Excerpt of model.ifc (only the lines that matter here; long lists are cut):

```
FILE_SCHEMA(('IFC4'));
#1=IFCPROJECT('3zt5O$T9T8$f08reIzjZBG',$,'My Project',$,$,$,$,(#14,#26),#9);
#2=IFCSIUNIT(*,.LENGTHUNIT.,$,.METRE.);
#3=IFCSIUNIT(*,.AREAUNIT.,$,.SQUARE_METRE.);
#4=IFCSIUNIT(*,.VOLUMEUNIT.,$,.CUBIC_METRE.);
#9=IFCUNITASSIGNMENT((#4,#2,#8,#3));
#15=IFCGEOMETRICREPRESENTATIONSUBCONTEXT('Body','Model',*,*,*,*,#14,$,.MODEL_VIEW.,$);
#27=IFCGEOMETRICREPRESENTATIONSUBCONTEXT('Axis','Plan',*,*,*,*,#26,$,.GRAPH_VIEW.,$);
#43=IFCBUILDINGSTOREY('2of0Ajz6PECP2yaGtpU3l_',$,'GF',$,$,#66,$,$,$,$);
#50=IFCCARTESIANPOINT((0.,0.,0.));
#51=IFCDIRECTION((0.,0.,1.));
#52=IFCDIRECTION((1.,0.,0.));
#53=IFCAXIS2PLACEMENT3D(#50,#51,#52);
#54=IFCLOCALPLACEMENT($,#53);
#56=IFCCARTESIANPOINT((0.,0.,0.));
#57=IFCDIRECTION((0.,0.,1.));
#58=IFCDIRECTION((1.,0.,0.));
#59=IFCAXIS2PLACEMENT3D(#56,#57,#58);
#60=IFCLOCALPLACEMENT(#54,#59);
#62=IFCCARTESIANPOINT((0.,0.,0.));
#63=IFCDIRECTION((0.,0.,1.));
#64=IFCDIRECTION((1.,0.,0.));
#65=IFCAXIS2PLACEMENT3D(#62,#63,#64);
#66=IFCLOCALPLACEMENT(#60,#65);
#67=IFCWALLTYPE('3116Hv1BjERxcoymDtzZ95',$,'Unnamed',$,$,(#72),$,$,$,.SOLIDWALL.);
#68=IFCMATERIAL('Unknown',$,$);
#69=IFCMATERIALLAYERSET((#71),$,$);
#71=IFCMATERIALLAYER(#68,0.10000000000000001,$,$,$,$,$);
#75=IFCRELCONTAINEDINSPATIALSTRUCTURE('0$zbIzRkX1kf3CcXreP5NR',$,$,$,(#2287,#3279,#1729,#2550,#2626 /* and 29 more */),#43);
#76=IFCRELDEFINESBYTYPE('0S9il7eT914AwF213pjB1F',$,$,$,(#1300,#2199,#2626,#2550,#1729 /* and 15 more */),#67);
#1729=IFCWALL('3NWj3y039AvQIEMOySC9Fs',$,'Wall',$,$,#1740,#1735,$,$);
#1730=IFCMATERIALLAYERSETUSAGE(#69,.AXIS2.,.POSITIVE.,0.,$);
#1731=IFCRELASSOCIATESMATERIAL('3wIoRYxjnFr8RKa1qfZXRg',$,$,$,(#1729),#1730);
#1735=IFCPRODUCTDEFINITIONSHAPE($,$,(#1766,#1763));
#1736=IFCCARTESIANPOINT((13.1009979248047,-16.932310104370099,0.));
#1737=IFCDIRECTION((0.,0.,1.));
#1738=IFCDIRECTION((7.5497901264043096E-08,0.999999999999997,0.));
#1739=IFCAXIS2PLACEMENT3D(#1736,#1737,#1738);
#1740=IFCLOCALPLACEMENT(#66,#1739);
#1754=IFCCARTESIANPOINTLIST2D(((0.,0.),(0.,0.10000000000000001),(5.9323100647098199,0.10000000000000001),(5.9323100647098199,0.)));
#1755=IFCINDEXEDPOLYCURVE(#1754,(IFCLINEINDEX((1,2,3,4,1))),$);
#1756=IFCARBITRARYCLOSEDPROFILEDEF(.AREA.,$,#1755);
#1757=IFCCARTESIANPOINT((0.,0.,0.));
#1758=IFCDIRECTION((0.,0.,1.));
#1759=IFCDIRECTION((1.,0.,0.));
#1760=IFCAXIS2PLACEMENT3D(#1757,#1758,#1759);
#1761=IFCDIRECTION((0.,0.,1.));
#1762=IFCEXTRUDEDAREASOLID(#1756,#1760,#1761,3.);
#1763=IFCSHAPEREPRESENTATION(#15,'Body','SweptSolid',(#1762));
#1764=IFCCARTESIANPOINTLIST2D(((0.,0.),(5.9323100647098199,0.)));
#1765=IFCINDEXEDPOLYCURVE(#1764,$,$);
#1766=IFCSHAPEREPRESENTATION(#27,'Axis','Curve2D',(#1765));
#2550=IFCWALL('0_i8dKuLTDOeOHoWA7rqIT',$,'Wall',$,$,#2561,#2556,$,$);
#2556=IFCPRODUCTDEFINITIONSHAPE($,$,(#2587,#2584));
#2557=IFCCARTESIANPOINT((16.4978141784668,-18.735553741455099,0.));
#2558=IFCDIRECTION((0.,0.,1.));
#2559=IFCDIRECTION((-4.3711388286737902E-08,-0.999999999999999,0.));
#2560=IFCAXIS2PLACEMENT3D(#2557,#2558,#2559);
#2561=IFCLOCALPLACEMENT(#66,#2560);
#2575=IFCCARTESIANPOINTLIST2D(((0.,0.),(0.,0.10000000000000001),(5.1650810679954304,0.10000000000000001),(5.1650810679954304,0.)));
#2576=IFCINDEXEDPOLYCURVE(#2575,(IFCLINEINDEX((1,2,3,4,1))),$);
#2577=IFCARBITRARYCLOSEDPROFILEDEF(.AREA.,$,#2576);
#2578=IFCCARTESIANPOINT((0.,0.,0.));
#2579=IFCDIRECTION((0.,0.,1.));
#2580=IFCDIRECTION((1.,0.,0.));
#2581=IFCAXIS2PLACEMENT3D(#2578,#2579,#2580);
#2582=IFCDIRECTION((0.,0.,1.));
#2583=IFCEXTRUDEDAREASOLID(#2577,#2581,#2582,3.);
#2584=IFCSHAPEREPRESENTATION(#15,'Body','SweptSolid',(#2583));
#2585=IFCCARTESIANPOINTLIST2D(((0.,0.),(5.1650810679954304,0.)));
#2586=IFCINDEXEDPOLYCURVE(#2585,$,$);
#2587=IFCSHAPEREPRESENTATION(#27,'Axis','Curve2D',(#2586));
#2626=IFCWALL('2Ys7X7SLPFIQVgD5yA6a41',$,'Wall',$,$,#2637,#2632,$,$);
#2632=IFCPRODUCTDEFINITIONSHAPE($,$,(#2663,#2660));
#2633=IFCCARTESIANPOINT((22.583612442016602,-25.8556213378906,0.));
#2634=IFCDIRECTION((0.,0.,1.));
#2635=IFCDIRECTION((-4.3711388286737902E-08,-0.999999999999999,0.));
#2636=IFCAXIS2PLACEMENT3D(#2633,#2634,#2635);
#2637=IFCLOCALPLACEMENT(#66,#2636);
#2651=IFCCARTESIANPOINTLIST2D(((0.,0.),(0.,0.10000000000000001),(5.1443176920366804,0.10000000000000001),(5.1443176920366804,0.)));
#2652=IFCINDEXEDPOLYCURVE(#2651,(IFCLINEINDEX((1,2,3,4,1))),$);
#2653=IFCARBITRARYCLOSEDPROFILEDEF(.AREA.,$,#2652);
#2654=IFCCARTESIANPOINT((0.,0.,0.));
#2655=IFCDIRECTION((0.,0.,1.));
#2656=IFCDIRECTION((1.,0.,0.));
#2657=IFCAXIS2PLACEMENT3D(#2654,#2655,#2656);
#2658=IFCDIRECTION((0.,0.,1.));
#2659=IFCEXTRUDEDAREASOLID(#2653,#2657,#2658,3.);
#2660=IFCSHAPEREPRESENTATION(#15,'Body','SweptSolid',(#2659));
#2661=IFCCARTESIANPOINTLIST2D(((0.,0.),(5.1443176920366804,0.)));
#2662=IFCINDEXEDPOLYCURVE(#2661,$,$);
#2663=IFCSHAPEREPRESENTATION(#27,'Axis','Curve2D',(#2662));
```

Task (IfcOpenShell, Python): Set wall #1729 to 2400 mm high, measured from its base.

```python
import ifcopenshell
import ifcopenshell.geom
import ifcopenshell.util.representation
import ifcopenshell.util.shape
import ifcopenshell.util.unit

model = ifcopenshell.open("model.ifc")
unit_scale = ifcopenshell.util.unit.calculate_unit_scale(model)
settings = ifcopenshell.geom.settings()


def volume(element):
    """Net volume in cubic metres, openings subtracted."""
    shape = ifcopenshell.geom.create_shape(settings, element)
    return ifcopenshell.util.shape.get_volume(shape.geometry)


wall = model.by_guid("3NWj3y039AvQIEMOySC9Fs")
before = volume(wall)

body = ifcopenshell.util.representation.get_representation(wall, "Model", "Body")
solid = body.Items[0]
old_height = solid.Depth
solid.Depth = 2.4 / unit_scale
after = volume(wall)

print(f"height {old_height:g} -> {solid.Depth:g}, volume {before:.3f} -> {after:.3f} m3")

model.write("model_updated.ifc")
```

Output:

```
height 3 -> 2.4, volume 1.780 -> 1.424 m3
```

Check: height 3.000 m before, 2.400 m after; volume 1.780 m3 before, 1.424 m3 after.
